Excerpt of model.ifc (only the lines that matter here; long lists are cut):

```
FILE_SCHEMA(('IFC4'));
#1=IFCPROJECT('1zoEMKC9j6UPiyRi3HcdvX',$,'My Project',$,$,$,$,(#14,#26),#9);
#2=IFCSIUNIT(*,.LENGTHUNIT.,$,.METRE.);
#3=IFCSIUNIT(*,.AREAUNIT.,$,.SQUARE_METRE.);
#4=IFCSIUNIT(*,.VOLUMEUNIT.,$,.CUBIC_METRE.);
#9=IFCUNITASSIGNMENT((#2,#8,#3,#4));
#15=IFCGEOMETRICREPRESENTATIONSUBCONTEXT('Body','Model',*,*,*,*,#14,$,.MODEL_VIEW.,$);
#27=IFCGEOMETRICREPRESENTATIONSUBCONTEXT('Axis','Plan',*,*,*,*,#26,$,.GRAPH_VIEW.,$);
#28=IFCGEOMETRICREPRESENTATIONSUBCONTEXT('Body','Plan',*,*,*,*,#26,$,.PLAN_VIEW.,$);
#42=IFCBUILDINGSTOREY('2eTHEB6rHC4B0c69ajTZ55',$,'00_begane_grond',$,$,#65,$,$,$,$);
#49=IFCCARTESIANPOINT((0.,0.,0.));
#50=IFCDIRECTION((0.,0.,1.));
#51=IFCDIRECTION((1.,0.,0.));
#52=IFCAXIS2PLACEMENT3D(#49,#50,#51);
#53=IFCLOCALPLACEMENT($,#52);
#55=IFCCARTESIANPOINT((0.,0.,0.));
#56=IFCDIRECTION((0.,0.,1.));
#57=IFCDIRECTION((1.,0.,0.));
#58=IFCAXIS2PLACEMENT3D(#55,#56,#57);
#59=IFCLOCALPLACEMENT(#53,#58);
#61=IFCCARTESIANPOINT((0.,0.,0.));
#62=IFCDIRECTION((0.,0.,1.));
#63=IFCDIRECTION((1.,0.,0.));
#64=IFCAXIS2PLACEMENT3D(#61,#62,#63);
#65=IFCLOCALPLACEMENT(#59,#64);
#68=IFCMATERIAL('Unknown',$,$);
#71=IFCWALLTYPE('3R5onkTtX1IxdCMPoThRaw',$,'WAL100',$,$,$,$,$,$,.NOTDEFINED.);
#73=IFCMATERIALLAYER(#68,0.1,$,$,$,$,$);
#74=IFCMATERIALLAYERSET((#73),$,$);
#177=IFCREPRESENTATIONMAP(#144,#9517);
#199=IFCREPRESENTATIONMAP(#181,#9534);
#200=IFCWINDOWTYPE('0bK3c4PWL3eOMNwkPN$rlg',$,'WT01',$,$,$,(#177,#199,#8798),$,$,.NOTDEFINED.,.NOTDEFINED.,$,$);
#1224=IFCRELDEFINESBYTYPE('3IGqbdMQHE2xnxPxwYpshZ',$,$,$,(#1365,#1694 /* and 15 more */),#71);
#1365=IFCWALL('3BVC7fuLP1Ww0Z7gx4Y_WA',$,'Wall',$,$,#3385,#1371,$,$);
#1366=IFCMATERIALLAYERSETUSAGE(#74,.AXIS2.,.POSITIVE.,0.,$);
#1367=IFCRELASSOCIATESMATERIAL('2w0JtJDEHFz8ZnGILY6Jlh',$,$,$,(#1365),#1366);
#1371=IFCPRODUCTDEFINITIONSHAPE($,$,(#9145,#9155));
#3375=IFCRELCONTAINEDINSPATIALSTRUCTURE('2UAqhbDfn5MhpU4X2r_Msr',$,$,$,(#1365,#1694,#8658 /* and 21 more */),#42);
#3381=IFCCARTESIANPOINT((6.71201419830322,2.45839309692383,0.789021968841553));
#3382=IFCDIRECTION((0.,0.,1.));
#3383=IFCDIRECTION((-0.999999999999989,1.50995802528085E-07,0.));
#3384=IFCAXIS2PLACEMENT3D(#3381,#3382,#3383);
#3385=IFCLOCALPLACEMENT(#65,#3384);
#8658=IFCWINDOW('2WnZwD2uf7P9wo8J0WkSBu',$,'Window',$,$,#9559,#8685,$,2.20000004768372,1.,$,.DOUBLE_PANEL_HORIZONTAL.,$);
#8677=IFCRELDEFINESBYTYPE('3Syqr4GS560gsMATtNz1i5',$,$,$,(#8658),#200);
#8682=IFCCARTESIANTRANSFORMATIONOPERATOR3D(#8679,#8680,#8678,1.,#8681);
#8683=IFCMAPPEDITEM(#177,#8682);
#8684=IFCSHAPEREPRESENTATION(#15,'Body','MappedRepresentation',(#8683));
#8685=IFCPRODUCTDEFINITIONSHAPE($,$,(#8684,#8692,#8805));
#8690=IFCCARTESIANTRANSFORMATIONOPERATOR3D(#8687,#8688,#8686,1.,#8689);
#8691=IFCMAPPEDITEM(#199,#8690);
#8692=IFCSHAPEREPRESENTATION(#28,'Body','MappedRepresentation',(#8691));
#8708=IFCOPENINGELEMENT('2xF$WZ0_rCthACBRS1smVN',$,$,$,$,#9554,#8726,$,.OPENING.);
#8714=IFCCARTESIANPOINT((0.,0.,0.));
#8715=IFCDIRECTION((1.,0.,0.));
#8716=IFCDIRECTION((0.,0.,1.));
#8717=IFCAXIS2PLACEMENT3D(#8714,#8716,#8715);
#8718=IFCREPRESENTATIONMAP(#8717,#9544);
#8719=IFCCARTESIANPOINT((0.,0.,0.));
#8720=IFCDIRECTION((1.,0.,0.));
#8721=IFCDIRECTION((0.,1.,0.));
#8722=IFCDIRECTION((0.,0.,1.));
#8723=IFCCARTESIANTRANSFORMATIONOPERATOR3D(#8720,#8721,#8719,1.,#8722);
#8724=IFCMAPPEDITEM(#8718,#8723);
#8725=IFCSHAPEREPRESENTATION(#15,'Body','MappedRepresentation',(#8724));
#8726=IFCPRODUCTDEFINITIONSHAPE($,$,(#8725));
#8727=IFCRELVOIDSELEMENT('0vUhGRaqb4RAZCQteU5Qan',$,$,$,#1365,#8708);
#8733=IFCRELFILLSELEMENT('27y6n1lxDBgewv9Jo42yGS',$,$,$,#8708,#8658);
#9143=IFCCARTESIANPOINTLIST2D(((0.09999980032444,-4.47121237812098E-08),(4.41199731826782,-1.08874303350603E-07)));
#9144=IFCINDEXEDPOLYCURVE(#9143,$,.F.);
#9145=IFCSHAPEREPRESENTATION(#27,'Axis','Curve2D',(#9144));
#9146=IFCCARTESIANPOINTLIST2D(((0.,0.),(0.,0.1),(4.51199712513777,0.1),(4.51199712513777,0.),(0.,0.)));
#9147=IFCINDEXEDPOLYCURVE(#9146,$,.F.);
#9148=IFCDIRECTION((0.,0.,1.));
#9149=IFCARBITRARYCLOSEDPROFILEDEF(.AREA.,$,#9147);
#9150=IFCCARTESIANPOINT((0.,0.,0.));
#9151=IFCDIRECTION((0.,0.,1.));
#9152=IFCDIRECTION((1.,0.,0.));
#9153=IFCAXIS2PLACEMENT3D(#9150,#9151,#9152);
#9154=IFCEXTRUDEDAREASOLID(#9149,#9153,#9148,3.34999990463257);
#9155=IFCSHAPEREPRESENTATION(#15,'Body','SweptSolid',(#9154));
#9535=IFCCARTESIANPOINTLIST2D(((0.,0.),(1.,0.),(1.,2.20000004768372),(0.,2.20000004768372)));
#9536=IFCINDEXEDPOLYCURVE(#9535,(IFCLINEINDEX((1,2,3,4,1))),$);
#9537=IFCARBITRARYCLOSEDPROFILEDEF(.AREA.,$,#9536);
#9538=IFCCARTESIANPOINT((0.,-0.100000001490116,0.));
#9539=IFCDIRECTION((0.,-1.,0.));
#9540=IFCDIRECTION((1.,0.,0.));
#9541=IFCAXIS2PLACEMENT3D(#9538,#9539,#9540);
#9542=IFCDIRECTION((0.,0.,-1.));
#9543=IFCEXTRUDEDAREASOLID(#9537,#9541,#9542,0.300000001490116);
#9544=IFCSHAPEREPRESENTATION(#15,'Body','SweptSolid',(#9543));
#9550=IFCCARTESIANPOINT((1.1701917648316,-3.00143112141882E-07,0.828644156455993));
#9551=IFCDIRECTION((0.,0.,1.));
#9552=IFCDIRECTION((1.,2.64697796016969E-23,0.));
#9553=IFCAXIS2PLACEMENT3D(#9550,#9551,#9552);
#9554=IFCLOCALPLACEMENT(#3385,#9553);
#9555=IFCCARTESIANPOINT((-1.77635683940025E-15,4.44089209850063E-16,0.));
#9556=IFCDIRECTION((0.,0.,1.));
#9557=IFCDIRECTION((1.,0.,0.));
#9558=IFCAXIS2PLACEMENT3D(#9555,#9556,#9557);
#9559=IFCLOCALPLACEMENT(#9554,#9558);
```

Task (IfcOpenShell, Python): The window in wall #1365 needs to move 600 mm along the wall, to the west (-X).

```python
import ifcopenshell
import ifcopenshell.api.geometry
import ifcopenshell.util.placement
import ifcopenshell.util.unit

model = ifcopenshell.open("model.ifc")
unit_scale = ifcopenshell.util.unit.calculate_unit_scale(model)

window = model.by_guid("2WnZwD2uf7P9wo8J0WkSBu")
opening = window.FillsVoids[0].RelatingOpeningElement
wall = opening.VoidsElements[0].RelatingBuildingElement

wall_matrix = ifcopenshell.util.placement.get_local_placement(wall.ObjectPlacement)
shift = wall_matrix[:3, 0] * 0.6 / unit_scale
before = ifcopenshell.util.placement.get_local_placement(window.ObjectPlacement)[:3, 3].copy()

# The window is placed relative to its opening, so it follows when the opening moves.
matrix = ifcopenshell.util.placement.get_local_placement(opening.ObjectPlacement)
matrix[:3, 3] += shift
ifcopenshell.api.geometry.edit_object_placement(
    model, product=opening, matrix=matrix, is_si=False, should_transform_children=True
)

after = ifcopenshell.util.placement.get_local_placement(window.ObjectPlacement)[:3, 3]
print("window moved by", (after - before).round(3) + 0.0)

model.write("model_rev.ifc")
```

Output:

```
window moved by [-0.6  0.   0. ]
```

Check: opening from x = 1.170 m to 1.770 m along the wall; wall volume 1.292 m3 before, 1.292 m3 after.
